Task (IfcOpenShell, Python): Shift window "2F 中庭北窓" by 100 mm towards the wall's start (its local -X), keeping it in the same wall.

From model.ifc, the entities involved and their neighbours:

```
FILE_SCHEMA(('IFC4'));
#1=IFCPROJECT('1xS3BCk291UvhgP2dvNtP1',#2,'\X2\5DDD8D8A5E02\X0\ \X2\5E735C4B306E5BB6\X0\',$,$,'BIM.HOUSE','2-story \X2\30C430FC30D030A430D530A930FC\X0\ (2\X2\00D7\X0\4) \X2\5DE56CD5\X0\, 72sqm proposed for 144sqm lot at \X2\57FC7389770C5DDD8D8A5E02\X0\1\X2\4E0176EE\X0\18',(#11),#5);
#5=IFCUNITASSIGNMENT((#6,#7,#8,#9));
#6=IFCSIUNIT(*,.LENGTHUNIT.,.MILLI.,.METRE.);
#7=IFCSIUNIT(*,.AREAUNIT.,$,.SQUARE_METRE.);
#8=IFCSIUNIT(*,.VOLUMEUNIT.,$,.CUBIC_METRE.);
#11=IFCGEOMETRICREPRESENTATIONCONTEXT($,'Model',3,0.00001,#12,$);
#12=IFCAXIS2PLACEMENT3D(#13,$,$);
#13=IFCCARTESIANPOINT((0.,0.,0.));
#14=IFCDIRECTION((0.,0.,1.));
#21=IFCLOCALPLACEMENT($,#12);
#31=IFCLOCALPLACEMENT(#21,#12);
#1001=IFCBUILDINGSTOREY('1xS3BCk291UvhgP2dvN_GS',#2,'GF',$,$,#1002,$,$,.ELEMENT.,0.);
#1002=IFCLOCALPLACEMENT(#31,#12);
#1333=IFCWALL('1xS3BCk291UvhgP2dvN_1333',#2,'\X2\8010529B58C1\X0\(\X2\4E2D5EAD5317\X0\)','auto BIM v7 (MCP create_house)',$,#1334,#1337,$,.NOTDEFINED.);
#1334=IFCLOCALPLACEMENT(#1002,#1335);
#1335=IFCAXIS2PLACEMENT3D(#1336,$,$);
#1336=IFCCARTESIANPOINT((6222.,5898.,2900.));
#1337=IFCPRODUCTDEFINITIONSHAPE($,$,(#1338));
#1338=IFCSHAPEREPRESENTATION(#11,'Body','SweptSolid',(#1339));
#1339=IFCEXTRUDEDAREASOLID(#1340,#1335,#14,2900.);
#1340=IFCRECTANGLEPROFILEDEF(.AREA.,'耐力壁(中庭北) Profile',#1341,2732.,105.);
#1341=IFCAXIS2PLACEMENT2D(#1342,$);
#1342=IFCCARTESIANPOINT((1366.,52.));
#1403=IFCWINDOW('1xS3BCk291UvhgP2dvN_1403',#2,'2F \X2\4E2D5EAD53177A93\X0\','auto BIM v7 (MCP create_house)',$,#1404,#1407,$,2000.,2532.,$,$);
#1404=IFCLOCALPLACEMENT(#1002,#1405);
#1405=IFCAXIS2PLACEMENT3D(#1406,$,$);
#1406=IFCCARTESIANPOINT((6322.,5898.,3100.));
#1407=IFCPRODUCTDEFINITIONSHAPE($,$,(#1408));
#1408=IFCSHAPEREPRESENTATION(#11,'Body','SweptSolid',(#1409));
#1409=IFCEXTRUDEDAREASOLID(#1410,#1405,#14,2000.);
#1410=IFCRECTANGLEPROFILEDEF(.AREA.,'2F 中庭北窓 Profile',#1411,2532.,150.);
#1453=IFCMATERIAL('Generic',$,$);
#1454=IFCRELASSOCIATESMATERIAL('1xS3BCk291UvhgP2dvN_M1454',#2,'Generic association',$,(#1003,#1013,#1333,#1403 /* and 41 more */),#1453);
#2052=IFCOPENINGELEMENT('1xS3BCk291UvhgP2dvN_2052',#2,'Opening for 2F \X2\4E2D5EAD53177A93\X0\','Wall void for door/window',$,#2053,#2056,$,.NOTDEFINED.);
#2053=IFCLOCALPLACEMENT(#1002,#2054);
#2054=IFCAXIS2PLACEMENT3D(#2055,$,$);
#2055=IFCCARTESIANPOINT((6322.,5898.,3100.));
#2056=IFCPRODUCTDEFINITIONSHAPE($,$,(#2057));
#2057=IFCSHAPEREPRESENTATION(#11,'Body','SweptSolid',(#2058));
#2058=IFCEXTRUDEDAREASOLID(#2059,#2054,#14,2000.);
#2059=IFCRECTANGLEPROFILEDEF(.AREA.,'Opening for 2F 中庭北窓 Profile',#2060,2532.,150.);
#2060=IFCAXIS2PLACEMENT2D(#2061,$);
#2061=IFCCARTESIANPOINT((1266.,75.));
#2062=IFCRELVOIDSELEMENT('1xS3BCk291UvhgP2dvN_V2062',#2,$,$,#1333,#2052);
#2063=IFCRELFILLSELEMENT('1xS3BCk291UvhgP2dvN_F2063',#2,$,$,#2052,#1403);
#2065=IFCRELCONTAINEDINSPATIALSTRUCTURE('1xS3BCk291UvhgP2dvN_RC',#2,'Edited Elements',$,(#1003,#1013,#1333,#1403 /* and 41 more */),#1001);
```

```python
import ifcopenshell
import ifcopenshell.api.geometry
import ifcopenshell.util.placement

model = ifcopenshell.open("model.ifc")

window = model.by_guid("1xS3BCk291UvhgP2dvN_1403")
opening = window.FillsVoids[0].RelatingOpeningElement
wall = opening.VoidsElements[0].RelatingBuildingElement

wall_matrix = ifcopenshell.util.placement.get_local_placement(wall.ObjectPlacement)
shift = wall_matrix[:3, 0] * -100.0
before = ifcopenshell.util.placement.get_local_placement(window.ObjectPlacement)[:3, 3].copy()

# The window is not placed relative to its opening, so move both.
for product in (opening, window):
    matrix = ifcopenshell.util.placement.get_local_placement(product.ObjectPlacement)
    matrix[:3, 3] += shift
    ifcopenshell.api.geometry.edit_object_placement(model, product=product, matrix=matrix, is_si=False)

after = ifcopenshell.util.placement.get_local_placement(window.ObjectPlacement)[:3, 3]
print("window moved by", (after - before).round(3) + 0.0)

model.write("model_edited.ifc")
```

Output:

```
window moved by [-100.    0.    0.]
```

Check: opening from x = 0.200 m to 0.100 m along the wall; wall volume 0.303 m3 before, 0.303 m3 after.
